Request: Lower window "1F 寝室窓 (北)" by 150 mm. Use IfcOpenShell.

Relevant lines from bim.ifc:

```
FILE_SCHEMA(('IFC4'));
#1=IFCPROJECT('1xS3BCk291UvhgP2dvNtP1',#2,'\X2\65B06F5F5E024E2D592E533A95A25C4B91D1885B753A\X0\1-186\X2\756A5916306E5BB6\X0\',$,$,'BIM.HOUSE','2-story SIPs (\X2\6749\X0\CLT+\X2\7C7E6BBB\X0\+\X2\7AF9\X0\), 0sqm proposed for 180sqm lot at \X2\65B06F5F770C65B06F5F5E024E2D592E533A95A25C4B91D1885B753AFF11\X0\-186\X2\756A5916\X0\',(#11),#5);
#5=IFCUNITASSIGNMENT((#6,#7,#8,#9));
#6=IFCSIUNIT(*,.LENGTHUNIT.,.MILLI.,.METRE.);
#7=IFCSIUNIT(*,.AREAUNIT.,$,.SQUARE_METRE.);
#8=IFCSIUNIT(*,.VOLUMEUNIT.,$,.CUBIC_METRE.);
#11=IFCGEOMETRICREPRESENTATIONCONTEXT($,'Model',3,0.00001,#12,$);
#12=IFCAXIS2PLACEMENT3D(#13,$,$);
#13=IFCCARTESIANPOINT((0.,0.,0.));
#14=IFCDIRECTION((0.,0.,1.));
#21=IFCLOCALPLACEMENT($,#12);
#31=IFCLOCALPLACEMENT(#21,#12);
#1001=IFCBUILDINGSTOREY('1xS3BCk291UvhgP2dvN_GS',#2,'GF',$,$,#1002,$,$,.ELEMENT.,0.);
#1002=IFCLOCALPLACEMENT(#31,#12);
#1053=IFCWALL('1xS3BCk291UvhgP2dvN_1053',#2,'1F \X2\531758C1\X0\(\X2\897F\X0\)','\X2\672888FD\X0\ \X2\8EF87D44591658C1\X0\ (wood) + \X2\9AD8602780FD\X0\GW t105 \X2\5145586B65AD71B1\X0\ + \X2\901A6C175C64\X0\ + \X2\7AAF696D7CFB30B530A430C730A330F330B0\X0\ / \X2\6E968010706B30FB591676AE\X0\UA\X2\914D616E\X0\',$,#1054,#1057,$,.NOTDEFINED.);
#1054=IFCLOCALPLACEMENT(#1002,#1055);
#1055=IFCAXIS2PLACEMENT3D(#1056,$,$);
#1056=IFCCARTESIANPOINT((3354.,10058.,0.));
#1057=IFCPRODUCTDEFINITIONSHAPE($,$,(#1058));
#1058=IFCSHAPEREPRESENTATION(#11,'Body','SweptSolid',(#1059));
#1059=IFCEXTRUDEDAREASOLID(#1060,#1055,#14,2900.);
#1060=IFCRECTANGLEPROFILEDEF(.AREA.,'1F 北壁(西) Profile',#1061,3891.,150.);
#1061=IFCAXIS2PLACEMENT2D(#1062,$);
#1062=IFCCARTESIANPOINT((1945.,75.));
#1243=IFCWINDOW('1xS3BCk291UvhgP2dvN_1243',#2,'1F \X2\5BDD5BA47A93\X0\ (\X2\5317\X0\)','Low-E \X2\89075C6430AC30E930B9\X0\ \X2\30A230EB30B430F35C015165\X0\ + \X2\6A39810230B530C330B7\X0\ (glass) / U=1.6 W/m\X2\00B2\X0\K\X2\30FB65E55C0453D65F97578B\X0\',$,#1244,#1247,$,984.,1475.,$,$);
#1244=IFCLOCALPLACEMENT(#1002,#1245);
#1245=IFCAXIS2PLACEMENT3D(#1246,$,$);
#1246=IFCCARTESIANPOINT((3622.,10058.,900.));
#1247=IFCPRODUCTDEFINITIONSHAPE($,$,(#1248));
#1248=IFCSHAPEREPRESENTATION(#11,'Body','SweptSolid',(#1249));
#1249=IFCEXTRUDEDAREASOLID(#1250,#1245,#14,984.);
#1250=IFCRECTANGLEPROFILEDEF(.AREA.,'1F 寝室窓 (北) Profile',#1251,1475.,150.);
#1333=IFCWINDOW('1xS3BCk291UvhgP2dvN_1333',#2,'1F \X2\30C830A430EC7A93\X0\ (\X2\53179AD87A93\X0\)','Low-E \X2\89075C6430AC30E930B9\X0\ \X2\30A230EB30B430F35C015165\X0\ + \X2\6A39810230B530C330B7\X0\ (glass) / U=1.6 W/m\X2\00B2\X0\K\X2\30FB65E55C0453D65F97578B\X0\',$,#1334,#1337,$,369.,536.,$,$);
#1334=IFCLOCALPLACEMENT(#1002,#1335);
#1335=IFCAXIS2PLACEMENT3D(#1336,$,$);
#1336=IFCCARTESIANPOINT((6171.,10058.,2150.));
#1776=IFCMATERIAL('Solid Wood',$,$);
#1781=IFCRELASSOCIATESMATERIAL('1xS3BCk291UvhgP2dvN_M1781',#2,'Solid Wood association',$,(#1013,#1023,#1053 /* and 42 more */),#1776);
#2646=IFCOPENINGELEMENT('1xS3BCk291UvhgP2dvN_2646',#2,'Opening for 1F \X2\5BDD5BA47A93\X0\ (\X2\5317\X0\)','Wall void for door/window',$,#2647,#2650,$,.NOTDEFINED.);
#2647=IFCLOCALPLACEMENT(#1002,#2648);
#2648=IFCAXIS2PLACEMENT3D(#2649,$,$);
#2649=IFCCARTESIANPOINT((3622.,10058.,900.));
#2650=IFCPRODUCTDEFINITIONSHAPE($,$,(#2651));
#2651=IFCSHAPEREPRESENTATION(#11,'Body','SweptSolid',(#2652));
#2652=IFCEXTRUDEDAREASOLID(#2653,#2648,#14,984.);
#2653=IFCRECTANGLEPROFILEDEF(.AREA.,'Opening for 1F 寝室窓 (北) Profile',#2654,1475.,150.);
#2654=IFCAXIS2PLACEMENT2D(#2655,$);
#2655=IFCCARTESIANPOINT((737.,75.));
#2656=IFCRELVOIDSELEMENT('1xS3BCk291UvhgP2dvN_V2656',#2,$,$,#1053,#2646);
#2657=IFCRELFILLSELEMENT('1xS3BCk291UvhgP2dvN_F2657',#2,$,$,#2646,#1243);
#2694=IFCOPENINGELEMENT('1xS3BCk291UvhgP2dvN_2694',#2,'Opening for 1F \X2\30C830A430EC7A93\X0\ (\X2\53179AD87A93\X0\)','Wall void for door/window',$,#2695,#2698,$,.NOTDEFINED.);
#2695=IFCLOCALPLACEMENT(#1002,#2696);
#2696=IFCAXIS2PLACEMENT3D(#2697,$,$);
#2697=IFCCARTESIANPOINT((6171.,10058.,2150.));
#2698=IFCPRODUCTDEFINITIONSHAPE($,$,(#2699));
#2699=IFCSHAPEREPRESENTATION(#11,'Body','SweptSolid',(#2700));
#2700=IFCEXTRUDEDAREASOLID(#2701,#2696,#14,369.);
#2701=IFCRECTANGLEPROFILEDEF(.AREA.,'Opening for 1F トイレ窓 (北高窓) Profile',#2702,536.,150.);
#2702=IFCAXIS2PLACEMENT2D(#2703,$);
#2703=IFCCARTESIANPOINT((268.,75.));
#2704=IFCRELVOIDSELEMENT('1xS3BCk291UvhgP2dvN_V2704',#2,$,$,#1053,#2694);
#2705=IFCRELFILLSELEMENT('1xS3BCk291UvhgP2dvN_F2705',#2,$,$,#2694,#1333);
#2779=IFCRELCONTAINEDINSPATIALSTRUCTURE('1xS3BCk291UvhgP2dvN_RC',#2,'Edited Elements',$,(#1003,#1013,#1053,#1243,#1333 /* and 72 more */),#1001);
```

```python
import numpy as np
import ifcopenshell
import ifcopenshell.api.geometry
import ifcopenshell.util.placement
import ifcopenshell.util.unit

model = ifcopenshell.open("bim.ifc")
unit_scale = ifcopenshell.util.unit.calculate_unit_scale(model)

window = model.by_id(1243)
opening = window.FillsVoids[0].RelatingOpeningElement
dz = -150.0

shift = np.array([0.0, 0.0, dz])
# The window is not placed relative to its opening, so move both.
for product in (opening, window):
    matrix = ifcopenshell.util.placement.get_local_placement(product.ObjectPlacement)
    matrix[:3, 3] += shift
    ifcopenshell.api.geometry.edit_object_placement(model, product=product, matrix=matrix, is_si=False)

print(f"moved by {dz * unit_scale:+.3f} m")

model.write("bim_updated.ifc")
```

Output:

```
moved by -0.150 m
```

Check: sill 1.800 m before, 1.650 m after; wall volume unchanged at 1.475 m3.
